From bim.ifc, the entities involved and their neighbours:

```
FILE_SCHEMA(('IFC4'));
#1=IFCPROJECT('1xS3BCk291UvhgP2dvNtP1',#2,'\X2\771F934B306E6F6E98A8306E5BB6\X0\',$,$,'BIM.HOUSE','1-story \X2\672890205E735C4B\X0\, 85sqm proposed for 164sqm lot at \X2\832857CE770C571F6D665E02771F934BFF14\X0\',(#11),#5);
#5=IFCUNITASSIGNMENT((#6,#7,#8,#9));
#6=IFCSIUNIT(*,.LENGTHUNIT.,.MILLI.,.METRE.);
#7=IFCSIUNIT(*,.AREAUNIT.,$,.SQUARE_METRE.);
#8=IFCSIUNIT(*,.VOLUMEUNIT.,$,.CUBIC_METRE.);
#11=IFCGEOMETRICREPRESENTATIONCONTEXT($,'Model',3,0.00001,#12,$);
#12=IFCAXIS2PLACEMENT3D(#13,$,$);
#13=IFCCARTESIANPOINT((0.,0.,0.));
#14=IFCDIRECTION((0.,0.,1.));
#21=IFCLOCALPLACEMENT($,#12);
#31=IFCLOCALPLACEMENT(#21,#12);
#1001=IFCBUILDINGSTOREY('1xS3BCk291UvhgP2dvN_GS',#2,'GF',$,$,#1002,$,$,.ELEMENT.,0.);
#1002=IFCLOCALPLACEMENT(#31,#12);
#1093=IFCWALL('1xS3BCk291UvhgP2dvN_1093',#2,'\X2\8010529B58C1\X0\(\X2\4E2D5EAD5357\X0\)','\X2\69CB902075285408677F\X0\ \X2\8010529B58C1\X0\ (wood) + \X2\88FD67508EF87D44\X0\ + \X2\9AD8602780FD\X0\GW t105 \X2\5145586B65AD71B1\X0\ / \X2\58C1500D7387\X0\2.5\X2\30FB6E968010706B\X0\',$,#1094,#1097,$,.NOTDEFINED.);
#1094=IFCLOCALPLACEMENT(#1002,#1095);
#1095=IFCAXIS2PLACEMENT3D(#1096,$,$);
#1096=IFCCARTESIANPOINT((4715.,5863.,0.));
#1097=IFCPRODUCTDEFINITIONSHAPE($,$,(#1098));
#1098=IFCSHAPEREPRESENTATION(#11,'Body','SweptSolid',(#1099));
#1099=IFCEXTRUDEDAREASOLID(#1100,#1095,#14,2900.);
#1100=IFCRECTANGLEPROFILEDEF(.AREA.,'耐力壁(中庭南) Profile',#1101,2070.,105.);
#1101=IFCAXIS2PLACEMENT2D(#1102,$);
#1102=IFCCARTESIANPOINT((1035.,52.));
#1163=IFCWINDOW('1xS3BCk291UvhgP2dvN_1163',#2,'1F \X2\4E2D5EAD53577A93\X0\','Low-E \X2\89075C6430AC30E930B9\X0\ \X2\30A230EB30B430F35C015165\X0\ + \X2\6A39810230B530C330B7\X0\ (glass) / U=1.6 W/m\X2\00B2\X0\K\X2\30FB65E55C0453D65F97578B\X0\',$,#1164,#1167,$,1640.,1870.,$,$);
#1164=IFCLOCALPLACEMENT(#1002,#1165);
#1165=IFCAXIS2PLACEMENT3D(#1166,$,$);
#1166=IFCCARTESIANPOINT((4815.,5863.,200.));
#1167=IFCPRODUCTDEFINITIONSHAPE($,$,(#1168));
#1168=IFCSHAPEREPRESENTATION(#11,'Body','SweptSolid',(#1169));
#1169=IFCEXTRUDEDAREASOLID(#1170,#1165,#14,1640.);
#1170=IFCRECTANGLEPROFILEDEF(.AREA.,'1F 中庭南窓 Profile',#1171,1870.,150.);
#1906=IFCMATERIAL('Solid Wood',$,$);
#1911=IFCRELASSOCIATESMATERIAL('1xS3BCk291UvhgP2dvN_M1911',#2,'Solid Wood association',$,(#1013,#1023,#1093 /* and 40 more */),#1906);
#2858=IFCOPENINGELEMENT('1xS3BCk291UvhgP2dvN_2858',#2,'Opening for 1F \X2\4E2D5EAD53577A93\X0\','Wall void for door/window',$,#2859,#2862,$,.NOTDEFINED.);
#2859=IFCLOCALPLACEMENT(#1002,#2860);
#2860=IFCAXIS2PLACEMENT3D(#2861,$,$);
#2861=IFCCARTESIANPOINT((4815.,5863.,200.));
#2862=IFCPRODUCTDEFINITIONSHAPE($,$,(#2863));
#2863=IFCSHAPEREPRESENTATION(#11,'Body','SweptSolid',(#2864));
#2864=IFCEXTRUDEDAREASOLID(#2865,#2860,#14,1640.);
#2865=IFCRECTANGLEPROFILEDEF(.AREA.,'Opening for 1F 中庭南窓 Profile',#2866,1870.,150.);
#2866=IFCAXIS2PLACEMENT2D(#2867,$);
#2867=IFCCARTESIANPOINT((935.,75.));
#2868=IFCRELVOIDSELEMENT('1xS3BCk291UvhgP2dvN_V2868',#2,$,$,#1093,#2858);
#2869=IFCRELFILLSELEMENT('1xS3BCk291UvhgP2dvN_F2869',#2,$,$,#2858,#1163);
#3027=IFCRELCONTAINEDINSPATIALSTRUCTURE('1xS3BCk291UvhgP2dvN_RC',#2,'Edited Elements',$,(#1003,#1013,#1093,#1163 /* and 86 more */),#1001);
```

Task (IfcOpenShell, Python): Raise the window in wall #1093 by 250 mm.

```python
import numpy as np
import ifcopenshell
import ifcopenshell.api.geometry
import ifcopenshell.util.placement
import ifcopenshell.util.unit

model = ifcopenshell.open("bim.ifc")
unit_scale = ifcopenshell.util.unit.calculate_unit_scale(model)

window = model.by_guid("1xS3BCk291UvhgP2dvN_1163")
opening = window.FillsVoids[0].RelatingOpeningElement
dz = 0.25 / unit_scale

shift = np.array([0.0, 0.0, dz])
# The window is not placed relative to its opening, so move both.
for product in (opening, window):
    matrix = ifcopenshell.util.placement.get_local_placement(product.ObjectPlacement)
    matrix[:3, 3] += shift
    ifcopenshell.api.geometry.edit_object_placement(model, product=product, matrix=matrix, is_si=False)

print(f"moved by {dz * unit_scale:+.3f} m")

model.write("bim_rev.ifc")
```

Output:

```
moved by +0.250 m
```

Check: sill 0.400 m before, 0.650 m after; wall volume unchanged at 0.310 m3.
